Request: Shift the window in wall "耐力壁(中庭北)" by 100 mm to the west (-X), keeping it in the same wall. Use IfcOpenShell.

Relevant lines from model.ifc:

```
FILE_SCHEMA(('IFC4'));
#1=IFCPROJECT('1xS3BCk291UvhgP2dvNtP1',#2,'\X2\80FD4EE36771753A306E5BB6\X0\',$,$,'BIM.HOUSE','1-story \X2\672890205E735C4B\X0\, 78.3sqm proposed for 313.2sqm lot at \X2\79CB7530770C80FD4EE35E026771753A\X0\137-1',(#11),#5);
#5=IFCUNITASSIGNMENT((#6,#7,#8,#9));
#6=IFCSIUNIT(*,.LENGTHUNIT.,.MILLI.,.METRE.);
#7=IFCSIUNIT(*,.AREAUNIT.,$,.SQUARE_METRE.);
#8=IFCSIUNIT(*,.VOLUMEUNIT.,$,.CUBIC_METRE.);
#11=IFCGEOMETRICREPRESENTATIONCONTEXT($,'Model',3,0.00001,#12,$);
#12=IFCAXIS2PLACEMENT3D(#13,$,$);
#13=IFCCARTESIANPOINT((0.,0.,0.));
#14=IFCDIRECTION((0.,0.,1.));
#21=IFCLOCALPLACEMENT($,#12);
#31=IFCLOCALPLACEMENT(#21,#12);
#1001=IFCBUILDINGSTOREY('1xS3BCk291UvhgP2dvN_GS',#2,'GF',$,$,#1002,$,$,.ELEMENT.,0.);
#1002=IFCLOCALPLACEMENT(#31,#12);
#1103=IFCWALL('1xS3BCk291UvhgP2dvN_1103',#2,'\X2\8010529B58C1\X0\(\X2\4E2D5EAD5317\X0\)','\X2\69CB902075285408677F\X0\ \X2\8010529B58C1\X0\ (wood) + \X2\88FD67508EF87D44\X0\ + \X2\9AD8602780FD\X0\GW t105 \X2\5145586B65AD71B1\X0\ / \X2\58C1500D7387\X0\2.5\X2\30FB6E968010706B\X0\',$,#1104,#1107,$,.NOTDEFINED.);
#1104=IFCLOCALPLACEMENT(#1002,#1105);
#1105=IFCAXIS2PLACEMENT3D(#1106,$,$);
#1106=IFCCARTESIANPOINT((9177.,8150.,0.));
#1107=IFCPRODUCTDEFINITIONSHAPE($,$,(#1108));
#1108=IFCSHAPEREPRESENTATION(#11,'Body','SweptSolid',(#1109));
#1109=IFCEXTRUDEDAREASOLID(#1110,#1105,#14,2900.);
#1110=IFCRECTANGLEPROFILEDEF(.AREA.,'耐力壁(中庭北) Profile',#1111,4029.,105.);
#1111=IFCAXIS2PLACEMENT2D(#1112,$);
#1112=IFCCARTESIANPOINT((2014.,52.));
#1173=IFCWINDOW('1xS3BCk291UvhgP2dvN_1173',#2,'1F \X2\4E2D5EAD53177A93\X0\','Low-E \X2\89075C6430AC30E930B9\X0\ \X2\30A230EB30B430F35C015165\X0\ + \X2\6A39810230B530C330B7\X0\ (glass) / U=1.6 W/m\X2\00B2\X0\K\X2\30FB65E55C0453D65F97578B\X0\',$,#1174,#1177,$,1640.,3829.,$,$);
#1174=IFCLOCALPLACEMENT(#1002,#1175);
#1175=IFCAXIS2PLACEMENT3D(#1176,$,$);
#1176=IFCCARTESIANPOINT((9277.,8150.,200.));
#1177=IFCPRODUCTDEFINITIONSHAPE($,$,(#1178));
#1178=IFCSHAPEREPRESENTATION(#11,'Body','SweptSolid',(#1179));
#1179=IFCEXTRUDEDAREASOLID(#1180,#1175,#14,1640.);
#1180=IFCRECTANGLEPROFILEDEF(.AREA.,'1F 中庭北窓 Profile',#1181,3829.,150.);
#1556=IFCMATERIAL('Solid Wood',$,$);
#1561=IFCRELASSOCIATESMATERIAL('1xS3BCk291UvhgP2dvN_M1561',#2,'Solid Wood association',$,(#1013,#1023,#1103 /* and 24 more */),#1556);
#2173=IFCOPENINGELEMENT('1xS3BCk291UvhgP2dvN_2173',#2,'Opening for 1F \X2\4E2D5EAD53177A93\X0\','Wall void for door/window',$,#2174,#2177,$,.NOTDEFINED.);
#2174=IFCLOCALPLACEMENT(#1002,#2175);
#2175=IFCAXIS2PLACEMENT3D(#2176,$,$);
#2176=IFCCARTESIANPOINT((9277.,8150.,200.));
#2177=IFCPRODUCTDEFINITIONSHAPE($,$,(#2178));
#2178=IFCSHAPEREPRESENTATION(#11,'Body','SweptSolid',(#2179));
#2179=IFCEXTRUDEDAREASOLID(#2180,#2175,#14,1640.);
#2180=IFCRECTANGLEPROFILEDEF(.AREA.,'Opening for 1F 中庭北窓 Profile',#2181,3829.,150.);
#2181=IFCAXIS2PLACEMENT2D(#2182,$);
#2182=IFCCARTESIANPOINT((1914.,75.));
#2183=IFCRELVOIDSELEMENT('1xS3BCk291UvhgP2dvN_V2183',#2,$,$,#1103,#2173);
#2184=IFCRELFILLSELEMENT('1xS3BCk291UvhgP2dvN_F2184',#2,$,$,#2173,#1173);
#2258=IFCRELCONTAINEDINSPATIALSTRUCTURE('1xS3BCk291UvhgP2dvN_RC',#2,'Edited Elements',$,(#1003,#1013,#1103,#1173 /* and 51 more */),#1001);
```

```python
import ifcopenshell
import ifcopenshell.api.geometry
import ifcopenshell.util.placement
import ifcopenshell.util.unit

model = ifcopenshell.open("model.ifc")
unit_scale = ifcopenshell.util.unit.calculate_unit_scale(model)

window = model.by_guid("1xS3BCk291UvhgP2dvN_1173")
opening = window.FillsVoids[0].RelatingOpeningElement
wall = opening.VoidsElements[0].RelatingBuildingElement

wall_matrix = ifcopenshell.util.placement.get_local_placement(wall.ObjectPlacement)
shift = wall_matrix[:3, 0] * -0.1 / unit_scale
before = ifcopenshell.util.placement.get_local_placement(window.ObjectPlacement)[:3, 3].copy()

# The window is not placed relative to its opening, so move both.
for product in (opening, window):
    matrix = ifcopenshell.util.placement.get_local_placement(product.ObjectPlacement)
    matrix[:3, 3] += shift
    ifcopenshell.api.geometry.edit_object_placement(model, product=product, matrix=matrix, is_si=False)

after = ifcopenshell.util.placement.get_local_placement(window.ObjectPlacement)[:3, 3]
print("window moved by", (after - before).round(3) + 0.0)

model.write("model_edited.ifc")
```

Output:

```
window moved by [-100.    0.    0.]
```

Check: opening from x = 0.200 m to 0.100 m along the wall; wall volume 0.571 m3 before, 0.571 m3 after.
